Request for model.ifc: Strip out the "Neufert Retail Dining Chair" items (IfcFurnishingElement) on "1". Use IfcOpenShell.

First a look at what the model holds.

```python
import ifcopenshell
import ifcopenshell.util.element

model = ifcopenshell.open("model.ifc")
print(model.schema)
storey = next(s for s in model.by_type("IfcBuildingStorey") if s.Name == "1")
furniture = [e for e in ifcopenshell.util.element.get_decomposition(storey) if e.is_a("IfcFurnishingElement")]
seen = {}
for e in furniture:
    element_type = ifcopenshell.util.element.get_type(e)
    name = element_type.Name if element_type not in (None, e) else None
    seen[name] = seen.get(name, 0) + 1
for name, count in sorted(seen.items(), key=str):
    print(count, "x", name)
```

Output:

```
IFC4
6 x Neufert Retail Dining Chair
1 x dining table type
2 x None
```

```python
import ifcopenshell
import ifcopenshell.api.root
import ifcopenshell.util.element

model = ifcopenshell.open("model.ifc")

storey = next(s for s in model.by_type("IfcBuildingStorey") if s.Name == "1")
furniture = [e for e in ifcopenshell.util.element.get_decomposition(storey) if e.is_a("IfcFurnishingElement")]
targets = [e for e in furniture if (t := ifcopenshell.util.element.get_type(e)) not in (None, e) and t.Name == "Neufert Retail Dining Chair"]

for e in targets:
    ifcopenshell.api.root.remove_product(model, product=e)
print(len(targets), "removed")

model.write("model_updated.ifc")
```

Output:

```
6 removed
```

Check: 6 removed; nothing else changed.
